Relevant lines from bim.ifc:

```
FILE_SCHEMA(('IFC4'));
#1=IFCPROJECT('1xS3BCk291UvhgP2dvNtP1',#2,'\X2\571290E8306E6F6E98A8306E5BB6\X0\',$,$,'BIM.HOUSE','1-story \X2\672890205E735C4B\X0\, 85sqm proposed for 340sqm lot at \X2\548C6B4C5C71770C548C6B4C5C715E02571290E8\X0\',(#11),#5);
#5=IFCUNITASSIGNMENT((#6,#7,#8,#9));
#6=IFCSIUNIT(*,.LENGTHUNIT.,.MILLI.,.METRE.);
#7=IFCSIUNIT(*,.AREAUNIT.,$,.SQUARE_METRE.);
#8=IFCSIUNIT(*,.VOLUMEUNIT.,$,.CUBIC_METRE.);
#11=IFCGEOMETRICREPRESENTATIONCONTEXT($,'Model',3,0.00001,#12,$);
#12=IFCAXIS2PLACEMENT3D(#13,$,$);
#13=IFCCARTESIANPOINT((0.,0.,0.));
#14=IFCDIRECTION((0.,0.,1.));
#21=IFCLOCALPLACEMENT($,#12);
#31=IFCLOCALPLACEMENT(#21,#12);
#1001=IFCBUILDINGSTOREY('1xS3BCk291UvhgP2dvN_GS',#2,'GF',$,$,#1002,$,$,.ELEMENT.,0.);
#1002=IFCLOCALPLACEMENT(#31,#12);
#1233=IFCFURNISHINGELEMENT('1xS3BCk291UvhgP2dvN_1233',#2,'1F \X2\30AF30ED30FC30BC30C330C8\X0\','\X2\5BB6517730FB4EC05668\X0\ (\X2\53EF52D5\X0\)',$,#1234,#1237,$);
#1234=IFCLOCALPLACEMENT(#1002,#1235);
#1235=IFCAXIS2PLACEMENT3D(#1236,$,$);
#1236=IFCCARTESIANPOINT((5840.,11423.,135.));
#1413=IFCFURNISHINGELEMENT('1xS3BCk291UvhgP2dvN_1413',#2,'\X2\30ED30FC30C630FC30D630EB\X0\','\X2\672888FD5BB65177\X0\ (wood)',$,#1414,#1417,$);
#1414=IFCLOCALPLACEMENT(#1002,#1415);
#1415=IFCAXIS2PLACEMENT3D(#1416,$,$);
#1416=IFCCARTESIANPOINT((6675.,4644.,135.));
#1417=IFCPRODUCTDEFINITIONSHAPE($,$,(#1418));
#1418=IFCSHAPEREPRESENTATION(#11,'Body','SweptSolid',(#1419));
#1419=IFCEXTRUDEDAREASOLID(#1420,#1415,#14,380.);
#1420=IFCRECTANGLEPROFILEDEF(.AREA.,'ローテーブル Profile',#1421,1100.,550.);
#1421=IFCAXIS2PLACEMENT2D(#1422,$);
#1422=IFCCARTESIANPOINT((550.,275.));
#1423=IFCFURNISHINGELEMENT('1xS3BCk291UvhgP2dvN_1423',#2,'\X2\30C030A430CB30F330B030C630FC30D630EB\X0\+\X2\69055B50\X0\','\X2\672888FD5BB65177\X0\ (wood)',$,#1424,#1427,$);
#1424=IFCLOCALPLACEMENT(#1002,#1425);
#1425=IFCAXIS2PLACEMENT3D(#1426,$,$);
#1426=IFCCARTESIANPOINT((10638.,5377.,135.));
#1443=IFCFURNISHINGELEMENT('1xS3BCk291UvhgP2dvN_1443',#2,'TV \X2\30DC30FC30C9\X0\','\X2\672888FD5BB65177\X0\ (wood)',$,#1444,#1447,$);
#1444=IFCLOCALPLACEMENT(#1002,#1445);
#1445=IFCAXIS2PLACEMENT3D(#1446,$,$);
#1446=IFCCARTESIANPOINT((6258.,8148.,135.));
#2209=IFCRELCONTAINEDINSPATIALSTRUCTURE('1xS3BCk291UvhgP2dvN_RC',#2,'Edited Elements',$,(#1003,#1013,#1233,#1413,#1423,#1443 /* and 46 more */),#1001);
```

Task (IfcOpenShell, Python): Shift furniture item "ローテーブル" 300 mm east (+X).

```python
import ifcopenshell
import ifcopenshell.api.geometry
import ifcopenshell.util.placement
import ifcopenshell.util.unit

model = ifcopenshell.open("bim.ifc")
unit_scale = ifcopenshell.util.unit.calculate_unit_scale(model)

item = model.by_guid("1xS3BCk291UvhgP2dvN_1413")
matrix = ifcopenshell.util.placement.get_local_placement(item.ObjectPlacement)
matrix[0, 3] += 0.3 / unit_scale
ifcopenshell.api.geometry.edit_object_placement(model, product=item, matrix=matrix, is_si=False)

print(ifcopenshell.util.placement.get_local_placement(item.ObjectPlacement).round(3) + 0.0)

model.write("bim_rev.ifc")
```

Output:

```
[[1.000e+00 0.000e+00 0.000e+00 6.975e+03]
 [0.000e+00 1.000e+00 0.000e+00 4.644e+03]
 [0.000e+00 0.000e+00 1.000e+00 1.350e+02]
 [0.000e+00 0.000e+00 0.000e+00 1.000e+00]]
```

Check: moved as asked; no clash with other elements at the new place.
